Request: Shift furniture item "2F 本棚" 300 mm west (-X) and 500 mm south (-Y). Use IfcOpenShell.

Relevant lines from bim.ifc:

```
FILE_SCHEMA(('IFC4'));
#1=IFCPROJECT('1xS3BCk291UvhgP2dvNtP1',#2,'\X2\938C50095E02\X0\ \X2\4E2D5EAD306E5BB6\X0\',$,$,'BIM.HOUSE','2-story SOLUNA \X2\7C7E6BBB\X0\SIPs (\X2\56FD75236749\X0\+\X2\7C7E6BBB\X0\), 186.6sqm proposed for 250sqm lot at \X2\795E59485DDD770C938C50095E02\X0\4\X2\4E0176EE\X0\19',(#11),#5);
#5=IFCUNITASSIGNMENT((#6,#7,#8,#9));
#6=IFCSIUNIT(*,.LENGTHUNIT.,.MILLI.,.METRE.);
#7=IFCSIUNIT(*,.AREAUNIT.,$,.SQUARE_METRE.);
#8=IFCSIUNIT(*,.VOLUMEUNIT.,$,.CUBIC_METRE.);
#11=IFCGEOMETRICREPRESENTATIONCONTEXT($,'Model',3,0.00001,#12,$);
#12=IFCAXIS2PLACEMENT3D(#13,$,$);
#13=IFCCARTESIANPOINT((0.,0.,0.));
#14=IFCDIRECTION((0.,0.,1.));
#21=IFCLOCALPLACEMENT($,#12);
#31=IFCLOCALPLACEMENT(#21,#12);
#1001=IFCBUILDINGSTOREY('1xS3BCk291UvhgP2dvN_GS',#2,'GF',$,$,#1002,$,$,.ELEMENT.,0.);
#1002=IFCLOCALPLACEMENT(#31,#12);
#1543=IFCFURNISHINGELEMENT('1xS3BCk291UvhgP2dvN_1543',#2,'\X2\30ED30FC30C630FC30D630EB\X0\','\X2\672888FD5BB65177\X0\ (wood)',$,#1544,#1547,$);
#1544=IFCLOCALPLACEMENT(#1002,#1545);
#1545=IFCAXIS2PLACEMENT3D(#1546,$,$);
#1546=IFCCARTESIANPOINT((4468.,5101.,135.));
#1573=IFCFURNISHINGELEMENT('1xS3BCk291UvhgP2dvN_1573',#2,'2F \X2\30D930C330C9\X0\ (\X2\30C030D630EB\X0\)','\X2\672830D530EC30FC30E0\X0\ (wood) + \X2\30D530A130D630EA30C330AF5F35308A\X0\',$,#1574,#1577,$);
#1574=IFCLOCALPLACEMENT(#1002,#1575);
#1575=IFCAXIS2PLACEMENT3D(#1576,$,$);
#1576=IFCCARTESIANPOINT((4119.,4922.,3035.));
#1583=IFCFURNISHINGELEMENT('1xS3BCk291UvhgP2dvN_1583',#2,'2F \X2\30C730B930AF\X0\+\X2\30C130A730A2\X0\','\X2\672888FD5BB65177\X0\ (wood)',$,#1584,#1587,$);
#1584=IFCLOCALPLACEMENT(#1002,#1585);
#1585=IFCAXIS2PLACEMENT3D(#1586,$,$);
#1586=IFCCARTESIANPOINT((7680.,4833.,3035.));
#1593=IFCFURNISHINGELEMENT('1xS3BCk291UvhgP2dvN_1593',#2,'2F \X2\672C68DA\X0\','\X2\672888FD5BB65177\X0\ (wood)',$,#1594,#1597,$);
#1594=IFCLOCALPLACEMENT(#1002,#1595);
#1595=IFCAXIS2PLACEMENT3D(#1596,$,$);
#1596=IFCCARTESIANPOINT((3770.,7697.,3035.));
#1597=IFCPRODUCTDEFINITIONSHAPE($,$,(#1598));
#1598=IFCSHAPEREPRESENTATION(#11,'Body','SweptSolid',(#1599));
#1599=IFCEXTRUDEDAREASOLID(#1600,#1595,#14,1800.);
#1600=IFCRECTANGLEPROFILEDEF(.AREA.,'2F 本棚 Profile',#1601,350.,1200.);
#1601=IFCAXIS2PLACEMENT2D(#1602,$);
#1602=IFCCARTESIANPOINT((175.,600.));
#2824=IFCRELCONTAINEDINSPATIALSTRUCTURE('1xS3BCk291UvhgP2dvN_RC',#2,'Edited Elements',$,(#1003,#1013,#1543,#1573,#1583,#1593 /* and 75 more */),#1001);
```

```python
import ifcopenshell
import ifcopenshell.api.geometry
import ifcopenshell.util.placement

model = ifcopenshell.open("bim.ifc")

item = model.by_id(1593)
matrix = ifcopenshell.util.placement.get_local_placement(item.ObjectPlacement)
matrix[0, 3] -= 300.0
matrix[1, 3] -= 500.0
ifcopenshell.api.geometry.edit_object_placement(model, product=item, matrix=matrix, is_si=False)

print(ifcopenshell.util.placement.get_local_placement(item.ObjectPlacement).round(3) + 0.0)

model.write("bim_rev.ifc")
```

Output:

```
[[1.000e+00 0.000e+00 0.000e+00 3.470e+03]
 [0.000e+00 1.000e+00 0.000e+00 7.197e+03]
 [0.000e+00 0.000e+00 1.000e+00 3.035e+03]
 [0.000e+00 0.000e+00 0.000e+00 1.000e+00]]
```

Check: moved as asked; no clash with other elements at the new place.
